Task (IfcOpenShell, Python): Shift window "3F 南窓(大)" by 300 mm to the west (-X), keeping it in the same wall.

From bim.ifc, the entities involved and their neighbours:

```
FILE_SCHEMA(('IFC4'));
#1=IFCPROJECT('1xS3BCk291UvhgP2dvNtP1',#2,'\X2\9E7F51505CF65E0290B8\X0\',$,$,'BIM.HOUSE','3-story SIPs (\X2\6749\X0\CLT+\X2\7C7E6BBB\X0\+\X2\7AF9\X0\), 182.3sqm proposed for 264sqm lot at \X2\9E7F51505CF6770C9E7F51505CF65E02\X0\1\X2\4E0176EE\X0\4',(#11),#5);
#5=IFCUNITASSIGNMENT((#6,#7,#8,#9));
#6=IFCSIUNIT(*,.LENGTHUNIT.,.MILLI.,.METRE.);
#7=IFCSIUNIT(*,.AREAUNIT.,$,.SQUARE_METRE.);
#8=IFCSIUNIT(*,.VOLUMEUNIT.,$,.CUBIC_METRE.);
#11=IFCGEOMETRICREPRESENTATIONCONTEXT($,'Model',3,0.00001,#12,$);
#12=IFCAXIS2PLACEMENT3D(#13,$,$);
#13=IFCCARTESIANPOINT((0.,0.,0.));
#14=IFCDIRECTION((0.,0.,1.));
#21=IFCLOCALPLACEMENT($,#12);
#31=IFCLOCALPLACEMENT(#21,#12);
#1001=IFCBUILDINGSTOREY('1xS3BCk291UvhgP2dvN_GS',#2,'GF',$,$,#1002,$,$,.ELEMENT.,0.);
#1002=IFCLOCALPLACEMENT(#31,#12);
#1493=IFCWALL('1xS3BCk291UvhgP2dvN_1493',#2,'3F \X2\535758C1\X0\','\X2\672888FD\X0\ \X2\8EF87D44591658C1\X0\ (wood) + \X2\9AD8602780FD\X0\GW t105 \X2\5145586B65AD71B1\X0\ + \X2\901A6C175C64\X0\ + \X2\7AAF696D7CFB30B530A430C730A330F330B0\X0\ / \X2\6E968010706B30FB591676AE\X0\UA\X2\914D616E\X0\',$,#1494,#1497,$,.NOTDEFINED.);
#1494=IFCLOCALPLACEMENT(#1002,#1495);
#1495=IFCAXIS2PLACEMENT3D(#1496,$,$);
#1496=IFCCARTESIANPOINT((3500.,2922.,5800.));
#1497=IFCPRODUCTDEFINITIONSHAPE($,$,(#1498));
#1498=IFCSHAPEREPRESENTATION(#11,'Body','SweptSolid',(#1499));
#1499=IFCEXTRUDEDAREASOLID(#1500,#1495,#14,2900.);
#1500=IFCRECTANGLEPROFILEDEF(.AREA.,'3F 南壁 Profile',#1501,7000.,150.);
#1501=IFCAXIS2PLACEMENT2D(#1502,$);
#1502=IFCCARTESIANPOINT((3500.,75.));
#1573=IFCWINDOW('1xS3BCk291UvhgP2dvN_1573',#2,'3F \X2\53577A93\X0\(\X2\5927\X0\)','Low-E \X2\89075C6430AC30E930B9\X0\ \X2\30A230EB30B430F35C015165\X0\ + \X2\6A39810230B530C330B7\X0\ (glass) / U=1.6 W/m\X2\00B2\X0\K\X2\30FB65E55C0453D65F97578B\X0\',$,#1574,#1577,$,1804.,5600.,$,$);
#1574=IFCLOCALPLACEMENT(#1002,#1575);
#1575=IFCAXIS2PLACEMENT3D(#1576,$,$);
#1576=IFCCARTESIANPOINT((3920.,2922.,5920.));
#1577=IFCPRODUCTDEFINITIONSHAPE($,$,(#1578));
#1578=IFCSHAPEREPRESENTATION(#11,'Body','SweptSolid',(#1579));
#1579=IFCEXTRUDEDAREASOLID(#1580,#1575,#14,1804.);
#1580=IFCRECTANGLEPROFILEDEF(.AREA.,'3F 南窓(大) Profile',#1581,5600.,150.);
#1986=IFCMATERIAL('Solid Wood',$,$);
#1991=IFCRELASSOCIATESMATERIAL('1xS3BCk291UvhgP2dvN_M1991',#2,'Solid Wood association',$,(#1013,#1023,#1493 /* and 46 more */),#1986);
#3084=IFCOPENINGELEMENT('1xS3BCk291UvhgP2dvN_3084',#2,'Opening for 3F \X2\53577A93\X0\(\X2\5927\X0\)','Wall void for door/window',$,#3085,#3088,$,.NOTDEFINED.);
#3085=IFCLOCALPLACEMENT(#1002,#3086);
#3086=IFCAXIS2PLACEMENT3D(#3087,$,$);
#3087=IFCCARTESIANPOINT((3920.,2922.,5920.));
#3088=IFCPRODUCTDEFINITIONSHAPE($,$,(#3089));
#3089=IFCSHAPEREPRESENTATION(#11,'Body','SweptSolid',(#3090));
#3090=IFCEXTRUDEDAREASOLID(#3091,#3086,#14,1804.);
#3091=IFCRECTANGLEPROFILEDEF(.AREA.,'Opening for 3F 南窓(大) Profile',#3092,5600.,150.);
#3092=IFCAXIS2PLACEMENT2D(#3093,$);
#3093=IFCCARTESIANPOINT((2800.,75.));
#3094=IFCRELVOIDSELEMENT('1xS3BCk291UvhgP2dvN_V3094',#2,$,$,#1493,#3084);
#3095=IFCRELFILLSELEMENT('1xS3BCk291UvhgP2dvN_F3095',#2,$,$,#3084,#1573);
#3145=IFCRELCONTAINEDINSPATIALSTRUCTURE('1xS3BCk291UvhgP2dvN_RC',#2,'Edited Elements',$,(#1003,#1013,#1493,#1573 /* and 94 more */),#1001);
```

```python
import ifcopenshell
import ifcopenshell.api.geometry
import ifcopenshell.util.placement
import ifcopenshell.util.unit

model = ifcopenshell.open("bim.ifc")
unit_scale = ifcopenshell.util.unit.calculate_unit_scale(model)

window = model.by_guid("1xS3BCk291UvhgP2dvN_1573")
opening = window.FillsVoids[0].RelatingOpeningElement
wall = opening.VoidsElements[0].RelatingBuildingElement

wall_matrix = ifcopenshell.util.placement.get_local_placement(wall.ObjectPlacement)
shift = wall_matrix[:3, 0] * -0.3 / unit_scale
before = ifcopenshell.util.placement.get_local_placement(window.ObjectPlacement)[:3, 3].copy()

# The window is not placed relative to its opening, so move both.
for product in (opening, window):
    matrix = ifcopenshell.util.placement.get_local_placement(product.ObjectPlacement)
    matrix[:3, 3] += shift
    ifcopenshell.api.geometry.edit_object_placement(model, product=product, matrix=matrix, is_si=False)

after = ifcopenshell.util.placement.get_local_placement(window.ObjectPlacement)[:3, 3]
print("window moved by", (after - before).round(3) + 0.0)

model.write("bim_v2.ifc")
```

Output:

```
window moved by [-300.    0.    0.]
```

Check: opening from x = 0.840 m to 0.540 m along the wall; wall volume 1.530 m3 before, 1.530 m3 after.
